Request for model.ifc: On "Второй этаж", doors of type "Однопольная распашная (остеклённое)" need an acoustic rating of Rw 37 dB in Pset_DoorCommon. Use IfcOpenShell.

First a look at what the model holds.

```python
import ifcopenshell
import ifcopenshell.util.element

model = ifcopenshell.open("model.ifc")
print(model.schema)
storey = next(s for s in model.by_type("IfcBuildingStorey") if s.Name == "Второй этаж")
doors = [e for e in ifcopenshell.util.element.get_decomposition(storey) if e.is_a("IfcDoor")]
seen = {}
for e in doors:
    element_type = ifcopenshell.util.element.get_type(e)
    key = (element_type.Name if element_type != e and element_type else None, ifcopenshell.util.element.get_pset(e, "Pset_DoorCommon", "AcousticRating"))
    seen[key] = seen.get(key, 0) + 1
for (name, value), count in sorted(seen.items(), key=str):
    print(count, "x", name, "|", value)
```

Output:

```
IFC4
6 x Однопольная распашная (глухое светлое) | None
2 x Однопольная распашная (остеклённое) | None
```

```python
import ifcopenshell
import ifcopenshell.api.pset
import ifcopenshell.util.element

model = ifcopenshell.open("model.ifc")

storey = next(s for s in model.by_type("IfcBuildingStorey") if s.Name == "Второй этаж")
doors = [e for e in ifcopenshell.util.element.get_decomposition(storey) if e.is_a("IfcDoor")]

count = 0
for e in doors:
    element_type = ifcopenshell.util.element.get_type(e)
    if element_type in (None, e) or element_type.Name != "Однопольная распашная (остеклённое)":
        continue
    # add_pset returns the element's existing set when there is one.
    pset = ifcopenshell.api.pset.add_pset(model, product=e, name="Pset_DoorCommon")
    ifcopenshell.api.pset.edit_pset(model, pset=pset, properties={"AcousticRating": "Rw 37 dB"})
    count += 1

print(count, "doors updated")

model.write("model_v2.ifc")
```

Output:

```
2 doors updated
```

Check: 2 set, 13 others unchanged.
